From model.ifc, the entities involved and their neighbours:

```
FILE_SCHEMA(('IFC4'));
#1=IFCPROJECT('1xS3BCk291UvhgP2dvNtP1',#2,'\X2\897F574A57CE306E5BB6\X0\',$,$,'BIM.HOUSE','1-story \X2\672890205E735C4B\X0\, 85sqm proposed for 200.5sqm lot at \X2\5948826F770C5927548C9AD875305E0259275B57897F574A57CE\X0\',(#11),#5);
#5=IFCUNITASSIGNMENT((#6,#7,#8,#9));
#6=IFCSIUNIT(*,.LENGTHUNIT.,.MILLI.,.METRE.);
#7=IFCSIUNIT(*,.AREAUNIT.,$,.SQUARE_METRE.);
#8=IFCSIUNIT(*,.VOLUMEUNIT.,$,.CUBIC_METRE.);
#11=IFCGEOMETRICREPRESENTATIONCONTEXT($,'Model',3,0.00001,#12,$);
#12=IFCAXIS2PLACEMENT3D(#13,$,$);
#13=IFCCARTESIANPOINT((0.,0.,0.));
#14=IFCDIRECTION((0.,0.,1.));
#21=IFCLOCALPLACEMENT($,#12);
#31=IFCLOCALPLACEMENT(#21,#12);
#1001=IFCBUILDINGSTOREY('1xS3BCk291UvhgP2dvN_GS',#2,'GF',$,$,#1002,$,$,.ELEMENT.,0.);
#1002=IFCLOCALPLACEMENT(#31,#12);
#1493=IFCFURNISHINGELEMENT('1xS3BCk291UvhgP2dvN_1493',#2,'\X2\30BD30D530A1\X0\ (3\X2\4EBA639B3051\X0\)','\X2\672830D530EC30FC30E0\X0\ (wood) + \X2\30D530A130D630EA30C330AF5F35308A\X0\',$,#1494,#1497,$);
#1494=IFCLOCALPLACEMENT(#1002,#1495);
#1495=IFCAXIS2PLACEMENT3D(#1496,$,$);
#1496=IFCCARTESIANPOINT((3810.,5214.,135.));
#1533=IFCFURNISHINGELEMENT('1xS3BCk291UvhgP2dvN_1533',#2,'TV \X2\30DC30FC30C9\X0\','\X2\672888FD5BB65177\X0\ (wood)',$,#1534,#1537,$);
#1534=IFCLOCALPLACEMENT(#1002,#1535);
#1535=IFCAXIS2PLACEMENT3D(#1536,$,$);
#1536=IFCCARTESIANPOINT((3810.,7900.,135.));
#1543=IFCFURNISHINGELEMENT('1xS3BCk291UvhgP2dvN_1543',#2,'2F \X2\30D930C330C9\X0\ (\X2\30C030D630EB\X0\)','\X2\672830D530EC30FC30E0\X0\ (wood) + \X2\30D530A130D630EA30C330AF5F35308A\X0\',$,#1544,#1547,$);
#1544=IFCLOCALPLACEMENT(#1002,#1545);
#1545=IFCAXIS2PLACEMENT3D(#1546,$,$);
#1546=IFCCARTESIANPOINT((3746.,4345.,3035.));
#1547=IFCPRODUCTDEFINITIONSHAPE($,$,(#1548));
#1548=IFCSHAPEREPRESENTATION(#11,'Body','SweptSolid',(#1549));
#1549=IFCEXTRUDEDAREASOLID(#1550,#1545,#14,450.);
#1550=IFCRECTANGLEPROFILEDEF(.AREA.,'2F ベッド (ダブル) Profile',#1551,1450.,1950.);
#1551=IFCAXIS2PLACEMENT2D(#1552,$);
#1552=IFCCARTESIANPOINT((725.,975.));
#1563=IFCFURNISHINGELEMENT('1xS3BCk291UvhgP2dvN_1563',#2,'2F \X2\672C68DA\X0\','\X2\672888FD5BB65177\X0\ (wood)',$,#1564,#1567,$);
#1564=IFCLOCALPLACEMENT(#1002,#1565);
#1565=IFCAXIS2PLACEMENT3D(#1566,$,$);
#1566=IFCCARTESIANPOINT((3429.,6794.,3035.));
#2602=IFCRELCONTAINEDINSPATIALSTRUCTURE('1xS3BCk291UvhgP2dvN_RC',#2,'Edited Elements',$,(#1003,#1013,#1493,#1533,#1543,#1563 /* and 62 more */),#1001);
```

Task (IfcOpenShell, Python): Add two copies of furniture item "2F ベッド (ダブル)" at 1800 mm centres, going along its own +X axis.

```python
import ifcopenshell
import ifcopenshell.api.geometry
import ifcopenshell.api.root
import ifcopenshell.util.element
import ifcopenshell.util.placement
import ifcopenshell.util.unit

model = ifcopenshell.open("model.ifc")
unit_scale = ifcopenshell.util.unit.calculate_unit_scale(model)


def reuse_history(source, copy):
    """copy_class also copies each property set's owner history, people and application; keep the originals."""
    for rel in copy.IsDefinedBy:
        if rel.is_a("IfcRelDefinesByProperties") and (history := rel.RelatingPropertyDefinition.OwnerHistory):
            rel.RelatingPropertyDefinition.OwnerHistory = source.OwnerHistory
            ifcopenshell.util.element.remove_deep2(model, history)


source = model.by_guid("1xS3BCk291UvhgP2dvN_1543")
base = ifcopenshell.util.placement.get_local_placement(source.ObjectPlacement)
step = base[:3, 0] * 1.8 / unit_scale

for i in range(1, 3):
    copy = ifcopenshell.api.root.copy_class(model, product=source)
    copy.Representation = ifcopenshell.util.element.copy_deep(
        model, source.Representation, exclude=["IfcGeometricRepresentationContext", "IfcRepresentationMap"]
    )
    reuse_history(source, copy)
    matrix = base.copy()
    matrix[:3, 3] += i * step
    print("added at", matrix[:3, 3].round(3) + 0.0)
    ifcopenshell.api.geometry.edit_object_placement(model, product=copy, matrix=matrix, is_si=False)

model.write("model_rev.ifc")
```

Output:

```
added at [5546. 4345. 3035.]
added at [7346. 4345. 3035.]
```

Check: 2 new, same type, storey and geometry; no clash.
